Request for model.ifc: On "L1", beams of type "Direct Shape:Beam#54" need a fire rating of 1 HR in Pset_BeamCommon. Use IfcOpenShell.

First a look at what the model holds.

```python
import ifcopenshell
import ifcopenshell.util.element

model = ifcopenshell.open("model.ifc")
print(model.schema)
storey = next(s for s in model.by_type("IfcBuildingStorey") if s.Name == "L1")
beams = [e for e in ifcopenshell.util.element.get_decomposition(storey) if e.is_a("IfcBeam")]
seen = {}
for e in beams:
    element_type = ifcopenshell.util.element.get_type(e)
    key = (element_type.Name if element_type != e and element_type else None, ifcopenshell.util.element.get_pset(e, "Pset_BeamCommon", "FireRating"))
    seen[key] = seen.get(key, 0) + 1
for (name, value), count in sorted(seen.items(), key=str):
    print(count, "x", name, "|", value)
```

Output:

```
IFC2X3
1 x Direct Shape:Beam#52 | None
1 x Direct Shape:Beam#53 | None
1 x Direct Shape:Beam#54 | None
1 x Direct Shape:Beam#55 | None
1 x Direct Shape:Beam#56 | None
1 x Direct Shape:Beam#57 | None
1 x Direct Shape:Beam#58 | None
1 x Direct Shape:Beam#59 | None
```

```python
import ifcopenshell
import ifcopenshell.api.pset
import ifcopenshell.util.element

model = ifcopenshell.open("model.ifc")

storey = next(s for s in model.by_type("IfcBuildingStorey") if s.Name == "L1")
beams = [e for e in ifcopenshell.util.element.get_decomposition(storey) if e.is_a("IfcBeam")]

count = 0
for e in beams:
    element_type = ifcopenshell.util.element.get_type(e)
    if element_type in (None, e) or element_type.Name != "Direct Shape:Beam#54":
        continue
    # add_pset returns the element's existing set when there is one.
    pset = ifcopenshell.api.pset.add_pset(model, product=e, name="Pset_BeamCommon")
    ifcopenshell.api.pset.edit_pset(model, pset=pset, properties={"FireRating": "1 HR"})
    count += 1

print(count, "beams updated")

model.write("model_rev.ifc")
```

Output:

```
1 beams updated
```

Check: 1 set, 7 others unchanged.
